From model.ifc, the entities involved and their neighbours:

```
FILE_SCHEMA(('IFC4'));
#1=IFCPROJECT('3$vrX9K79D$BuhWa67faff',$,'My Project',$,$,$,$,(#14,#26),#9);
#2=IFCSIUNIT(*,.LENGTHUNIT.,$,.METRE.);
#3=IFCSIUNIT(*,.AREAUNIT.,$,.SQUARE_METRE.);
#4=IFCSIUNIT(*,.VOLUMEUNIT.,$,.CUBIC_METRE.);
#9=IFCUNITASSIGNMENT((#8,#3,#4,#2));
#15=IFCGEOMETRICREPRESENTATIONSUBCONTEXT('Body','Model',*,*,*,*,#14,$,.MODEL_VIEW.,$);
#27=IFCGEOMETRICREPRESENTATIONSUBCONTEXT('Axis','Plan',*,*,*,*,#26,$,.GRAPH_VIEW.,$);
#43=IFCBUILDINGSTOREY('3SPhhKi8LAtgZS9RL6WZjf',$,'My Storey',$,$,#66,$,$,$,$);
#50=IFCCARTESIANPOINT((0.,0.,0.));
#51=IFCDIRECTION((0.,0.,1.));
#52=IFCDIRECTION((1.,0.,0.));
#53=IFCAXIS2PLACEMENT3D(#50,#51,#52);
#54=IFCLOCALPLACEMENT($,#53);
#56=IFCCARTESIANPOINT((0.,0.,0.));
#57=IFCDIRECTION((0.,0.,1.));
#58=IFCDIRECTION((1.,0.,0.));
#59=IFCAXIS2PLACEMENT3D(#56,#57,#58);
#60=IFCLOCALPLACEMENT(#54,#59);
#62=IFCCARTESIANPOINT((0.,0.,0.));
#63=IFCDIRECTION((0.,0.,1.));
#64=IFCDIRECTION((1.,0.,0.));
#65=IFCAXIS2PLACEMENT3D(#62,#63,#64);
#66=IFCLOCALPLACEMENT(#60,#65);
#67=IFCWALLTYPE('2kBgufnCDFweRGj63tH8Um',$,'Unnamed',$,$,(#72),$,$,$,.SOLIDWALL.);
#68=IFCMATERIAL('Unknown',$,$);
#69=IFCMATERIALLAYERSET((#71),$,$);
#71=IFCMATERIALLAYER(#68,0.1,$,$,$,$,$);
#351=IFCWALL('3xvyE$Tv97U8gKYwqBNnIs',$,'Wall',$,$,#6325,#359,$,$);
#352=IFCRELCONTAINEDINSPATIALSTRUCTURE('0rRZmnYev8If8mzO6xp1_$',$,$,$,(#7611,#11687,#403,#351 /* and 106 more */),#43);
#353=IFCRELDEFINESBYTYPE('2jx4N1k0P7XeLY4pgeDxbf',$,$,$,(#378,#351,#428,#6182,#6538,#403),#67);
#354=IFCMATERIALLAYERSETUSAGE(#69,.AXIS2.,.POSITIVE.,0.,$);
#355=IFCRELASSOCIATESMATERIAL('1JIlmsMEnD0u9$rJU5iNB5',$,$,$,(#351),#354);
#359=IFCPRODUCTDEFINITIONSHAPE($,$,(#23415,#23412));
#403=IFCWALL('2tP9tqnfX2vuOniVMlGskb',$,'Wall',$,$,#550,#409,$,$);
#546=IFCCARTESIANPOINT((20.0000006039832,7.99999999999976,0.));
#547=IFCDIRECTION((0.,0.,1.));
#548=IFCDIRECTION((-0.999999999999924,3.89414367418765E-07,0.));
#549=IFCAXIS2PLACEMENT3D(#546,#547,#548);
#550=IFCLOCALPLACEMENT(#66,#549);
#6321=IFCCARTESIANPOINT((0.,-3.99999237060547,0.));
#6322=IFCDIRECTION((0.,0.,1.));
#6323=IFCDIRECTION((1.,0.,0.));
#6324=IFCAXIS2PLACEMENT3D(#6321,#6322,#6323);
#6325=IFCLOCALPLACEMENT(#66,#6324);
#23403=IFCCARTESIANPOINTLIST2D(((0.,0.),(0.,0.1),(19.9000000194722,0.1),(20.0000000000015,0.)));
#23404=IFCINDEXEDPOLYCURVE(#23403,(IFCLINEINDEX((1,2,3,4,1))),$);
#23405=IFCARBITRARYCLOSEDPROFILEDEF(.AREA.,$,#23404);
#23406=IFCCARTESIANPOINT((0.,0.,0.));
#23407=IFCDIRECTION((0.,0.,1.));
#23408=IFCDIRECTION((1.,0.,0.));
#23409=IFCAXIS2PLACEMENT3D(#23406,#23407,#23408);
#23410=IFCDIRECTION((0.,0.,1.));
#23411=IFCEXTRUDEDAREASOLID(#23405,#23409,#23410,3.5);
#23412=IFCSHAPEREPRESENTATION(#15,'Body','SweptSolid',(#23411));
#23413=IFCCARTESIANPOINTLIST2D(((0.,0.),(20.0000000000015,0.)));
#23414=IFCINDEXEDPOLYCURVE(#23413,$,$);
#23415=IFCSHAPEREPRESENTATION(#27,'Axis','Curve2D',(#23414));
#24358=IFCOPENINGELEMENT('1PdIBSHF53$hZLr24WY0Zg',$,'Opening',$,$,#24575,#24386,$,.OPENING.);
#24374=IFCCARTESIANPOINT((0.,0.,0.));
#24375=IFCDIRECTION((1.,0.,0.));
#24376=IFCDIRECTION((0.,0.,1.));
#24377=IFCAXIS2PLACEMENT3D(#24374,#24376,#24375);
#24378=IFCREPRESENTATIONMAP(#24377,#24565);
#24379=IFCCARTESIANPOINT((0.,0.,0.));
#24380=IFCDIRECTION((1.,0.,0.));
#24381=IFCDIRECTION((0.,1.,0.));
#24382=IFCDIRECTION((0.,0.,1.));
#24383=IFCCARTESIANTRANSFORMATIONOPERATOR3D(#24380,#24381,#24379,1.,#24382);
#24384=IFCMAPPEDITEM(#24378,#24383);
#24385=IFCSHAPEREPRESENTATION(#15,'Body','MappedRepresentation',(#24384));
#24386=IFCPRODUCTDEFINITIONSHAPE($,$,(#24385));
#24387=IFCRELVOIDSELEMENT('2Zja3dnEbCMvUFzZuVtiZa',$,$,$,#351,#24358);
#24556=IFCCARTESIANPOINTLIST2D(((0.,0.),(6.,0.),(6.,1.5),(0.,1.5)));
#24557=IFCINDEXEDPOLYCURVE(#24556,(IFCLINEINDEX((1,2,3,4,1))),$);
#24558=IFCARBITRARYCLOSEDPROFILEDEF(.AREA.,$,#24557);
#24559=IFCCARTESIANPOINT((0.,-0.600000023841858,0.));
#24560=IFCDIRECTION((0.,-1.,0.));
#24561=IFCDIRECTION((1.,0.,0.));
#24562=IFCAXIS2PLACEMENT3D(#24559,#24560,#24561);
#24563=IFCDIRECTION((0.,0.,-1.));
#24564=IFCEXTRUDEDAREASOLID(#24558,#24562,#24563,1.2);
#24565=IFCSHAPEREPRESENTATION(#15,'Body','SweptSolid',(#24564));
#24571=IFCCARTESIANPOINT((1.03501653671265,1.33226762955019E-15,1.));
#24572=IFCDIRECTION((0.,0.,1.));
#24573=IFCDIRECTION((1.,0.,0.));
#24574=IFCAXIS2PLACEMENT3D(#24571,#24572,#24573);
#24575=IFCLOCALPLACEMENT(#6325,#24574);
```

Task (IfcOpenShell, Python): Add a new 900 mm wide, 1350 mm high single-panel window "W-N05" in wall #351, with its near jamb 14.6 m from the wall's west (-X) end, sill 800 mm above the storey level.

```python
import numpy as np
import ifcopenshell
import ifcopenshell.api.feature
import ifcopenshell.api.geometry
import ifcopenshell.api.root
import ifcopenshell.api.spatial
import ifcopenshell.geom
import ifcopenshell.util.element
import ifcopenshell.util.placement
import ifcopenshell.util.representation
import ifcopenshell.util.shape
import ifcopenshell.util.unit

model = ifcopenshell.open("model.ifc")
unit_scale = ifcopenshell.util.unit.calculate_unit_scale(model)
settings = ifcopenshell.geom.settings()


def volume(element):
    """Net volume in cubic metres, openings subtracted."""
    shape = ifcopenshell.geom.create_shape(settings, element)
    return ifcopenshell.util.shape.get_volume(shape.geometry)


wall = model.by_id(351)
storey = ifcopenshell.util.element.get_container(wall, ifc_class="IfcBuildingStorey")
context = ifcopenshell.util.representation.get_context(model, "Model", "Body", "MODEL_VIEW")
before = volume(wall)

width, height, from_end, sill = 0.9, 1.35, 14.6, 0.8  # metres

# The wall runs along its own X axis, and the end named is its -X end.
wall_shape = ifcopenshell.geom.create_shape(settings, wall)
x, y, z = ifcopenshell.util.shape.get_vertices(wall_shape.geometry).T
start = x.min() + from_end
face, thickness = float(y.min()), float(y.max() - y.min())
wall_matrix = ifcopenshell.util.placement.get_local_placement(wall.ObjectPlacement)
level = ifcopenshell.util.placement.get_local_placement(storey.ObjectPlacement)[2, 3]


def in_wall(x, y):
    """Placement at x, y metres in the wall's axes, at sill height."""
    matrix = wall_matrix.copy()
    matrix[:, 3] = wall_matrix @ np.array([x / unit_scale, y / unit_scale, 0.0, 1.0])
    matrix[2, 3] = level + sill / unit_scale
    return matrix


# Opening: a box that overshoots both wall faces by 50 mm.
opening = ifcopenshell.api.root.create_entity(model, ifc_class="IfcOpeningElement", predefined_type="OPENING")
box = ifcopenshell.api.geometry.add_wall_representation(
    model, context=context, length=width, height=height, thickness=thickness + 0.1
)
ifcopenshell.api.geometry.assign_representation(model, product=opening, representation=box)
ifcopenshell.api.geometry.edit_object_placement(model, product=opening, matrix=in_wall(start, face - 0.05), is_si=False)
ifcopenshell.api.feature.add_feature(model, feature=opening, element=wall)

window = ifcopenshell.api.root.create_entity(model, ifc_class="IfcWindow", name="W-N05", predefined_type="WINDOW")
window.OverallWidth, window.OverallHeight = width / unit_scale, height / unit_scale
window.PartitioningType = "SINGLE_PANEL"
body = ifcopenshell.api.geometry.add_window_representation(
    model,
    context=context,
    overall_width=window.OverallWidth,
    overall_height=window.OverallHeight,
    partition_type="SINGLE_PANEL",
)
ifcopenshell.api.geometry.assign_representation(model, product=window, representation=body)
ifcopenshell.api.spatial.assign_container(model, products=[window], relating_structure=storey)
ifcopenshell.api.feature.add_filling(model, opening=opening, element=window)

# Centre the window in the wall's thickness.
ifcopenshell.api.geometry.edit_object_placement(model, product=window, matrix=in_wall(start, face), is_si=False)
window_shape = ifcopenshell.geom.create_shape(settings, window)
depth = ifcopenshell.util.shape.get_vertices(window_shape.geometry)[:, 1]
offset = face + thickness / 2 - (depth.min() + depth.max()) / 2
ifcopenshell.api.geometry.edit_object_placement(model, product=window, matrix=in_wall(start, offset), is_si=False)

after = volume(wall)

print(f"wall volume {before:.3f} -> {after:.3f} m3")

model.write("model_rev.ifc")
```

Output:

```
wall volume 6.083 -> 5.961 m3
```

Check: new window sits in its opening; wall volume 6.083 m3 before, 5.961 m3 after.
